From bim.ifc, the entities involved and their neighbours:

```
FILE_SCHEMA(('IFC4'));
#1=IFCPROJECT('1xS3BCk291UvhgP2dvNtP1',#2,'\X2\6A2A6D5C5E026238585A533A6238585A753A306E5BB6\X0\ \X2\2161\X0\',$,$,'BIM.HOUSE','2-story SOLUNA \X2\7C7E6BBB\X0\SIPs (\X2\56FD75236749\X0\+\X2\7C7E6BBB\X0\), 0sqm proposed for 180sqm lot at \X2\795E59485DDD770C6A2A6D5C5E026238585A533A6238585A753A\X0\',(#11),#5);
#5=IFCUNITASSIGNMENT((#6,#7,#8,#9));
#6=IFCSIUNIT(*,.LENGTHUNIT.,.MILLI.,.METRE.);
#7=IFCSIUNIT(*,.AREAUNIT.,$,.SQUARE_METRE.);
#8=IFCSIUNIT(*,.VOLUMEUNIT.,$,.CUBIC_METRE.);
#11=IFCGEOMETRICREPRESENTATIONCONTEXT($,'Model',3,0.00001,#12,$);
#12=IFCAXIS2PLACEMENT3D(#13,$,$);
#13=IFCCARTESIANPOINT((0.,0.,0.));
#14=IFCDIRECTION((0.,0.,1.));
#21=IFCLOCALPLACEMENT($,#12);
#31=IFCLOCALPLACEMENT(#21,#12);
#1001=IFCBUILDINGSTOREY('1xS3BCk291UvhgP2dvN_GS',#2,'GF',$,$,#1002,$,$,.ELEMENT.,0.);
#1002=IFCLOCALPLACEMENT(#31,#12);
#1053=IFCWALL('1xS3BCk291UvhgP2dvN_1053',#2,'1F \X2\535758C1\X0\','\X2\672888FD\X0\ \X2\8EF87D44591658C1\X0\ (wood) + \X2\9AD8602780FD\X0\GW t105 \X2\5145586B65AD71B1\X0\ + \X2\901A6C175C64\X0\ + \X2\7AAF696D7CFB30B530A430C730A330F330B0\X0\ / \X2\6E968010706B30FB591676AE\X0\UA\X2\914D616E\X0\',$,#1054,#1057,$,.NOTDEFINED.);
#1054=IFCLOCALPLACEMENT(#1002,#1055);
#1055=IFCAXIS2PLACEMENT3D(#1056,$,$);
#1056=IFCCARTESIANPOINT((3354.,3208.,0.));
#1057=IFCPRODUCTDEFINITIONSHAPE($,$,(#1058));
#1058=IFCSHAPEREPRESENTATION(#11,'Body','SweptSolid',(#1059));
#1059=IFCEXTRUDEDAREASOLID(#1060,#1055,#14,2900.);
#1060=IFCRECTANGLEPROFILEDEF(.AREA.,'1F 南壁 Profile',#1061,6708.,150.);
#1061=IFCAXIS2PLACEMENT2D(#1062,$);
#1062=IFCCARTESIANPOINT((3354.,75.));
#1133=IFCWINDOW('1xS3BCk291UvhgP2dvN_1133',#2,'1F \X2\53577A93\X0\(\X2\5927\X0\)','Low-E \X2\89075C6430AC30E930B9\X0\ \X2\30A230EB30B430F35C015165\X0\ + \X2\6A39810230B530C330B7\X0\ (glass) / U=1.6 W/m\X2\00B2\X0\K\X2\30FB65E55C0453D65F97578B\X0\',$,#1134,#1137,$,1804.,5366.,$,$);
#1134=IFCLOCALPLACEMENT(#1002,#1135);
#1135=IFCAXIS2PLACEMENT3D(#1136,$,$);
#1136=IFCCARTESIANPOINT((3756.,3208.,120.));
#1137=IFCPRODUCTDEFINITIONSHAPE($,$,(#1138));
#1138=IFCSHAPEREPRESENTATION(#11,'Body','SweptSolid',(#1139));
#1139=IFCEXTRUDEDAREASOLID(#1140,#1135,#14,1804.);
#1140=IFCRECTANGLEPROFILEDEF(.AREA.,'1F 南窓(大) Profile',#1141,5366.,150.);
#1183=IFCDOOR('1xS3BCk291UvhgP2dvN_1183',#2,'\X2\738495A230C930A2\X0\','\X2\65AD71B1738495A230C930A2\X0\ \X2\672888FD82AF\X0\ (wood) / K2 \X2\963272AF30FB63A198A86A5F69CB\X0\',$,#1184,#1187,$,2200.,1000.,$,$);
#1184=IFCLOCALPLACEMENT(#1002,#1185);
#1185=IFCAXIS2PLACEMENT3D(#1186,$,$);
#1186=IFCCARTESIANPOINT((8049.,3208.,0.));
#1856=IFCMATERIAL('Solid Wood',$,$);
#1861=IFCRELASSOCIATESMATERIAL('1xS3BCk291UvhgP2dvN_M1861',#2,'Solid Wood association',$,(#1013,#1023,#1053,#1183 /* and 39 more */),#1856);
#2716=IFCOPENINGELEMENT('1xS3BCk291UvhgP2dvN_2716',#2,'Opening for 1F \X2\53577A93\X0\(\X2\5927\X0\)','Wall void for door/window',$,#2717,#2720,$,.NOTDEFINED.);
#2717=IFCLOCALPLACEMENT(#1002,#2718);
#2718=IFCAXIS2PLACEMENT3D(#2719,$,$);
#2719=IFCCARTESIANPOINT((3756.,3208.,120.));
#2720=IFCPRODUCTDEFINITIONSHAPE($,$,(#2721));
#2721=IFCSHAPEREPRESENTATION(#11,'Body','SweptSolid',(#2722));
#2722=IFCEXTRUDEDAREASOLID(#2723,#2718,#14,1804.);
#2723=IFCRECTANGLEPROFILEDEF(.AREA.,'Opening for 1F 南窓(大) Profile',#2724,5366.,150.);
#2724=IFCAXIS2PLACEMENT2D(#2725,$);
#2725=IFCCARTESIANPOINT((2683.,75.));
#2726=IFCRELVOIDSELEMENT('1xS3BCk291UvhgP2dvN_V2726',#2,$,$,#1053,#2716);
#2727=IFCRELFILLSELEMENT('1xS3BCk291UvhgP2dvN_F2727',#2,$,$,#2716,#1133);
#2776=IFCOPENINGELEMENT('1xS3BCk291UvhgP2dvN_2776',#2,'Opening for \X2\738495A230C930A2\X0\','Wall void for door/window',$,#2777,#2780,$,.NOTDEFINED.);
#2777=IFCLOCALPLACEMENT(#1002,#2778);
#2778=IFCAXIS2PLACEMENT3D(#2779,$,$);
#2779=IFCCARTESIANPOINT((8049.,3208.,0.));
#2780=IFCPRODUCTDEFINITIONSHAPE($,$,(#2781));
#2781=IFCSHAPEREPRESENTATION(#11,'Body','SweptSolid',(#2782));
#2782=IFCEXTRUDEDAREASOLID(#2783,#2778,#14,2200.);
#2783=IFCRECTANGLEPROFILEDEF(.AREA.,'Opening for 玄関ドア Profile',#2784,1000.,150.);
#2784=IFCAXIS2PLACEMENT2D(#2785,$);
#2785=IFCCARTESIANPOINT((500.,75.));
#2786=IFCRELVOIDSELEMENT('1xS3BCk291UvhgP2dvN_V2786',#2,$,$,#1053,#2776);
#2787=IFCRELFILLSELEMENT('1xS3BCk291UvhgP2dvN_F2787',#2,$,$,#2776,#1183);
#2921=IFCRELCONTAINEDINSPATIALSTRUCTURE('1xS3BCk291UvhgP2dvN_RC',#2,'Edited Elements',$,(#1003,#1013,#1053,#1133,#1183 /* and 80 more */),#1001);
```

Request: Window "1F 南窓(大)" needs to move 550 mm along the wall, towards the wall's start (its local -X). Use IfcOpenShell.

```python
import ifcopenshell
import ifcopenshell.api.geometry
import ifcopenshell.util.placement
import ifcopenshell.util.unit

model = ifcopenshell.open("bim.ifc")
unit_scale = ifcopenshell.util.unit.calculate_unit_scale(model)

window = model.by_id(1133)
opening = window.FillsVoids[0].RelatingOpeningElement
wall = opening.VoidsElements[0].RelatingBuildingElement

wall_matrix = ifcopenshell.util.placement.get_local_placement(wall.ObjectPlacement)
shift = wall_matrix[:3, 0] * -0.55 / unit_scale
before = ifcopenshell.util.placement.get_local_placement(window.ObjectPlacement)[:3, 3].copy()

# The window is not placed relative to its opening, so move both.
for product in (opening, window):
    matrix = ifcopenshell.util.placement.get_local_placement(product.ObjectPlacement)
    matrix[:3, 3] += shift
    ifcopenshell.api.geometry.edit_object_placement(model, product=product, matrix=matrix, is_si=False)

after = ifcopenshell.util.placement.get_local_placement(window.ObjectPlacement)[:3, 3]
print("window moved by", (after - before).round(3) + 0.0)

model.write("bim_rev.ifc")
```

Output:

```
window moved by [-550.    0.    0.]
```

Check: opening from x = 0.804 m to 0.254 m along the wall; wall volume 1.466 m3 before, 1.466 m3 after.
